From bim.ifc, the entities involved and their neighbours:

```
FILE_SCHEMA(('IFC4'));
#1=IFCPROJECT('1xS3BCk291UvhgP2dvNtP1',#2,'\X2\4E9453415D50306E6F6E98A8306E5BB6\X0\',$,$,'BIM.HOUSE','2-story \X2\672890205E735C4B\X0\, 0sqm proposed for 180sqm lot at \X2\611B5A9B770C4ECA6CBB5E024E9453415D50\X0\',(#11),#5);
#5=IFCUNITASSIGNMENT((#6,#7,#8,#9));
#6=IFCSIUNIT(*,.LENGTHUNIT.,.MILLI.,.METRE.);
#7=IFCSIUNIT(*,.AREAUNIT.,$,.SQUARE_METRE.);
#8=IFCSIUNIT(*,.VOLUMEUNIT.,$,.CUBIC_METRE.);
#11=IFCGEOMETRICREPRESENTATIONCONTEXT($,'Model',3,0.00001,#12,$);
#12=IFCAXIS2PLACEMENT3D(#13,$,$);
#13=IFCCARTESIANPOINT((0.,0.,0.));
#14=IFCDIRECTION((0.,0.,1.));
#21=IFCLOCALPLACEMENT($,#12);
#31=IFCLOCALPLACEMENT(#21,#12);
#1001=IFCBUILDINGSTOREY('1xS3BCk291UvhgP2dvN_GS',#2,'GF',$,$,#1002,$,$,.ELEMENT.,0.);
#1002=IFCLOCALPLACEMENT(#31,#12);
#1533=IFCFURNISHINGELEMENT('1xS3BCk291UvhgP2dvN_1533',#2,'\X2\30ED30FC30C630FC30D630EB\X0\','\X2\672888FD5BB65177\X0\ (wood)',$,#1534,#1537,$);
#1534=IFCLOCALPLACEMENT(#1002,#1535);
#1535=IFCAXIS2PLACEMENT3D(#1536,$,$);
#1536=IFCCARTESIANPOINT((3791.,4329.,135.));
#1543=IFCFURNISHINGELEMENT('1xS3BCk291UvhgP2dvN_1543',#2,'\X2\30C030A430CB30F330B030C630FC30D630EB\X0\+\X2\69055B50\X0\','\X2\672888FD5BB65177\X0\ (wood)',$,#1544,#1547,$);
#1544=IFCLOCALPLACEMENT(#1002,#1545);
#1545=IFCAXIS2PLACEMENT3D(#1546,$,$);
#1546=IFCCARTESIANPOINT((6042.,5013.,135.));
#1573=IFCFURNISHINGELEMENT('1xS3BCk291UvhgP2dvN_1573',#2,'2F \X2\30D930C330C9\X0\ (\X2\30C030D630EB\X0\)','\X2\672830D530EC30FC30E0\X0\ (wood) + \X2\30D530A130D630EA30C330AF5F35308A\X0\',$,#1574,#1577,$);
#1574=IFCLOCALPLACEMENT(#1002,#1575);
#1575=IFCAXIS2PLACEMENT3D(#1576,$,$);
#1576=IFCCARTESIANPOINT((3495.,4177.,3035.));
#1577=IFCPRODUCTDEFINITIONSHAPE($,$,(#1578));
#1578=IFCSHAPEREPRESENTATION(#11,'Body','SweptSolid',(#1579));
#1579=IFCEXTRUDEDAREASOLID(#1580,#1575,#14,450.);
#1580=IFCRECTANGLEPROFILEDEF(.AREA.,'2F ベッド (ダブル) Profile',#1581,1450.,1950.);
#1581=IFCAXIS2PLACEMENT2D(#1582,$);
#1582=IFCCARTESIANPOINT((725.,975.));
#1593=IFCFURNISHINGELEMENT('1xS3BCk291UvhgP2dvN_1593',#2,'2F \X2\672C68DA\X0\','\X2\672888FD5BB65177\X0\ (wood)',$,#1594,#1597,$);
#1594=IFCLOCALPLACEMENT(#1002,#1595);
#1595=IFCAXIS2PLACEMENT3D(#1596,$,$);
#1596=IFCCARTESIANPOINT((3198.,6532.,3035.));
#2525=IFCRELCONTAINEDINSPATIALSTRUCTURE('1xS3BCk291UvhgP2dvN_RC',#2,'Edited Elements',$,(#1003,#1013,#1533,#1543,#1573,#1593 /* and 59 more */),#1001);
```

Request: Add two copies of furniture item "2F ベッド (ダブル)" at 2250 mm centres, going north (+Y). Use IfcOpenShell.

```python
import numpy as np
import ifcopenshell
import ifcopenshell.api.geometry
import ifcopenshell.api.root
import ifcopenshell.util.element
import ifcopenshell.util.placement
import ifcopenshell.util.unit

model = ifcopenshell.open("bim.ifc")
unit_scale = ifcopenshell.util.unit.calculate_unit_scale(model)


def reuse_history(source, copy):
    """copy_class also copies each property set's owner history, people and application; keep the originals."""
    for rel in copy.IsDefinedBy:
        if rel.is_a("IfcRelDefinesByProperties") and (history := rel.RelatingPropertyDefinition.OwnerHistory):
            rel.RelatingPropertyDefinition.OwnerHistory = source.OwnerHistory
            ifcopenshell.util.element.remove_deep2(model, history)


source = model.by_id(1573)
base = ifcopenshell.util.placement.get_local_placement(source.ObjectPlacement)
step = np.array([0.0, 1.0, 0.0]) * 2.25 / unit_scale

for i in range(1, 3):
    copy = ifcopenshell.api.root.copy_class(model, product=source)
    copy.Representation = ifcopenshell.util.element.copy_deep(
        model, source.Representation, exclude=["IfcGeometricRepresentationContext", "IfcRepresentationMap"]
    )
    reuse_history(source, copy)
    matrix = base.copy()
    matrix[:3, 3] += i * step
    print("added at", matrix[:3, 3].round(3) + 0.0)
    ifcopenshell.api.geometry.edit_object_placement(model, product=copy, matrix=matrix, is_si=False)

model.write("bim_updated.ifc")
```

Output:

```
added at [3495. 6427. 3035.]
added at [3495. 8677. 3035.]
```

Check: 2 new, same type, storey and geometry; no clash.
